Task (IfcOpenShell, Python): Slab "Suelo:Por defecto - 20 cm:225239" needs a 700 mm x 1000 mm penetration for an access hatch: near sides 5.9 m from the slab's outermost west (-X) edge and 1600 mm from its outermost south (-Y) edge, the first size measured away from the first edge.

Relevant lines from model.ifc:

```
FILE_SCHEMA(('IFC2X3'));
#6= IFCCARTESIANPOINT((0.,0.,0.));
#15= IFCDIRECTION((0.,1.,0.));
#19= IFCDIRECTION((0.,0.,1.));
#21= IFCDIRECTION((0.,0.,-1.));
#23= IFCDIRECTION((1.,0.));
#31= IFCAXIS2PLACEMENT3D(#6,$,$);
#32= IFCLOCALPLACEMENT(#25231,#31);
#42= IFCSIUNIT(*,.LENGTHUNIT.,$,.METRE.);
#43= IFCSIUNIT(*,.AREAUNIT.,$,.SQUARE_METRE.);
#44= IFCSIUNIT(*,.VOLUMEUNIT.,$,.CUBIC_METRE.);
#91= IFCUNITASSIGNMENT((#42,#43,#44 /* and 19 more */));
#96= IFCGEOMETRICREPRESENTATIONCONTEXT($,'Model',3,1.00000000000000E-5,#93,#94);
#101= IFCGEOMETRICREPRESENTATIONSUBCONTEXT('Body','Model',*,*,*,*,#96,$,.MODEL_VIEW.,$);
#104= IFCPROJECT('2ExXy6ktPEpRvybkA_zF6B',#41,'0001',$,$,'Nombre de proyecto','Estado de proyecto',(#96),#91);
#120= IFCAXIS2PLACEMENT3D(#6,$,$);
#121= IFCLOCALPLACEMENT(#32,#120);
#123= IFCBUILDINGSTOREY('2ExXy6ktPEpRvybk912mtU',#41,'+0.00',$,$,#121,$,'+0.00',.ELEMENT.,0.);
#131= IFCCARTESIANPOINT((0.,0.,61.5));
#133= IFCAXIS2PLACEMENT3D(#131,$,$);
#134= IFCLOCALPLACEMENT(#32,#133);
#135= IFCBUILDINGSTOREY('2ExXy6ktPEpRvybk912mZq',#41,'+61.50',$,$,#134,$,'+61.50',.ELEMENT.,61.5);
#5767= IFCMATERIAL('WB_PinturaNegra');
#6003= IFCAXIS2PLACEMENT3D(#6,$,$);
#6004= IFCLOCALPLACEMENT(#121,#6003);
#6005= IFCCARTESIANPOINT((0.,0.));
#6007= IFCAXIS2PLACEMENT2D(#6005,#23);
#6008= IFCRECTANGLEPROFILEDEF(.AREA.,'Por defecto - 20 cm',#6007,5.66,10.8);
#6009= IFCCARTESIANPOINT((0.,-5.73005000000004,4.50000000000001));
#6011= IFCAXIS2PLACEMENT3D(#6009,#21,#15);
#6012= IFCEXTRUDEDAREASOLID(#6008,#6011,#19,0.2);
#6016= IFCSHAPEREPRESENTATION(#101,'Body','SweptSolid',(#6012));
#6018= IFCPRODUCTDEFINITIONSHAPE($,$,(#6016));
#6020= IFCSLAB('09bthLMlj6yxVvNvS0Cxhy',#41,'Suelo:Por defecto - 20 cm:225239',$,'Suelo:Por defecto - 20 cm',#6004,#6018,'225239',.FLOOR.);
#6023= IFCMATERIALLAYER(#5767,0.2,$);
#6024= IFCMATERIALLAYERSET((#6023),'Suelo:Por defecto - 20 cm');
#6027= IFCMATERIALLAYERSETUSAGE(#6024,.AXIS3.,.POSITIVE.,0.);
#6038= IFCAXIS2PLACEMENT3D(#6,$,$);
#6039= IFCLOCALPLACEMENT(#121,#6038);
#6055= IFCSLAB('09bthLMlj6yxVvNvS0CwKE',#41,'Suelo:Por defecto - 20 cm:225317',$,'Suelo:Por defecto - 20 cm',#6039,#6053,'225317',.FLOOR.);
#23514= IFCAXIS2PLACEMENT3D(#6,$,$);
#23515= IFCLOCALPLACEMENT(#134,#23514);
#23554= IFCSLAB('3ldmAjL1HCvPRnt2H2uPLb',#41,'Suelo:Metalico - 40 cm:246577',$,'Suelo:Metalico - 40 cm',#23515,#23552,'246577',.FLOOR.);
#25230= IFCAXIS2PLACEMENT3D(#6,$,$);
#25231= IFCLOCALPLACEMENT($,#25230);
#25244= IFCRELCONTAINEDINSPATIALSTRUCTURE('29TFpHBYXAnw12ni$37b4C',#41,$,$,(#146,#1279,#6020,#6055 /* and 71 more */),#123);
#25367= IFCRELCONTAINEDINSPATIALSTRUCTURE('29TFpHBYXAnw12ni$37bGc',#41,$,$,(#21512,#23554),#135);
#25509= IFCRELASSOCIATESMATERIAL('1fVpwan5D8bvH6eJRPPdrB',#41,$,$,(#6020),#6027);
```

```python
import numpy as np
import ifcopenshell
import ifcopenshell.api.feature
import ifcopenshell.api.geometry
import ifcopenshell.api.root
import ifcopenshell.geom
import ifcopenshell.util.placement
import ifcopenshell.util.representation
import ifcopenshell.util.shape
import ifcopenshell.util.unit

model = ifcopenshell.open("model.ifc")
unit_scale = ifcopenshell.util.unit.calculate_unit_scale(model)
settings = ifcopenshell.geom.settings()


def volume(element):
    """Net volume in cubic metres, openings subtracted."""
    shape = ifcopenshell.geom.create_shape(settings, element)
    return ifcopenshell.util.shape.get_volume(shape.geometry)


slab = model.by_guid("09bthLMlj6yxVvNvS0Cxhy")
before = volume(slab)

# Extent in the slab's own axes, in metres. The edges named are its -X and -Y sides.
slab_shape = ifcopenshell.geom.create_shape(settings, slab)
vertices = ifcopenshell.util.shape.get_vertices(slab_shape.geometry)
x_min, y_min, bottom = vertices.min(axis=0)
top = vertices[:, 2].max()

opening = ifcopenshell.api.root.create_entity(model, ifc_class="IfcOpeningElement", name="Access hatch opening")
context = ifcopenshell.util.representation.get_context(model, "Model", "Body", "MODEL_VIEW")
width, depth = 0.7, 1
outline = [(0.0, 0.0), (width, 0.0), (width, depth), (0.0, depth), (0.0, 0.0)]
# Overshoot both faces by 50 mm so the cut is clean.
shape = ifcopenshell.api.geometry.add_slab_representation(
    model, context=context, depth=top - bottom + 0.1, polyline=outline
)
ifcopenshell.api.geometry.assign_representation(model, product=opening, representation=shape)

matrix = ifcopenshell.util.placement.get_local_placement(slab.ObjectPlacement)
matrix[:, 3] = matrix @ np.append(np.array([x_min + 5.9, y_min + 1.6, bottom - 0.05]) / unit_scale, 1.0)
ifcopenshell.api.geometry.edit_object_placement(model, product=opening, matrix=matrix, is_si=False)
ifcopenshell.api.feature.add_feature(model, feature=opening, element=slab)

after = volume(slab)

print(f"slab volume {before:.3f} -> {after:.3f} m3")

model.write("model_rev.ifc")
```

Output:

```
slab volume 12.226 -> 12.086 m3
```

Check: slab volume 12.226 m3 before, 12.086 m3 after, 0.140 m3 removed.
